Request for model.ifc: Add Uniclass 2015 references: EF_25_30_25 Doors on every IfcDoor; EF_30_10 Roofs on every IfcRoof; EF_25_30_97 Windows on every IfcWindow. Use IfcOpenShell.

First a look at what the model holds.

```python
import ifcopenshell

model = ifcopenshell.open("model.ifc")
print(model.schema)
print("classifications:", [c.Name for c in model.by_type("IfcClassification")])
for ifc_class in ("IfcDoor", "IfcRoof", "IfcStair", "IfcWall", "IfcWindow"):
    print(ifc_class, len(model.by_type(ifc_class)))
```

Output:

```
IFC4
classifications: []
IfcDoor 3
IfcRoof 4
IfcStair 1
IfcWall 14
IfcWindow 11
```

```python
import ifcopenshell
import ifcopenshell.api.classification

model = ifcopenshell.open("model.ifc")

system = ifcopenshell.api.classification.add_classification(model, classification="Uniclass 2015")

codes = {
    "IfcDoor": ("EF_25_30_25", "Doors"),
    "IfcRoof": ("EF_30_10", "Roofs"),
    "IfcWindow": ("EF_25_30_97", "Windows"),
}
for ifc_class, (code, name) in codes.items():
    products = model.by_type(ifc_class)
    ifcopenshell.api.classification.add_reference(
        model, products=products, classification=system, identification=code, name=name
    )
    print(code, len(products))

model.write("model_v2.ifc")
```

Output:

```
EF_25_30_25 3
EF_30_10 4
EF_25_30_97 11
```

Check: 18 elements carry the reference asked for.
